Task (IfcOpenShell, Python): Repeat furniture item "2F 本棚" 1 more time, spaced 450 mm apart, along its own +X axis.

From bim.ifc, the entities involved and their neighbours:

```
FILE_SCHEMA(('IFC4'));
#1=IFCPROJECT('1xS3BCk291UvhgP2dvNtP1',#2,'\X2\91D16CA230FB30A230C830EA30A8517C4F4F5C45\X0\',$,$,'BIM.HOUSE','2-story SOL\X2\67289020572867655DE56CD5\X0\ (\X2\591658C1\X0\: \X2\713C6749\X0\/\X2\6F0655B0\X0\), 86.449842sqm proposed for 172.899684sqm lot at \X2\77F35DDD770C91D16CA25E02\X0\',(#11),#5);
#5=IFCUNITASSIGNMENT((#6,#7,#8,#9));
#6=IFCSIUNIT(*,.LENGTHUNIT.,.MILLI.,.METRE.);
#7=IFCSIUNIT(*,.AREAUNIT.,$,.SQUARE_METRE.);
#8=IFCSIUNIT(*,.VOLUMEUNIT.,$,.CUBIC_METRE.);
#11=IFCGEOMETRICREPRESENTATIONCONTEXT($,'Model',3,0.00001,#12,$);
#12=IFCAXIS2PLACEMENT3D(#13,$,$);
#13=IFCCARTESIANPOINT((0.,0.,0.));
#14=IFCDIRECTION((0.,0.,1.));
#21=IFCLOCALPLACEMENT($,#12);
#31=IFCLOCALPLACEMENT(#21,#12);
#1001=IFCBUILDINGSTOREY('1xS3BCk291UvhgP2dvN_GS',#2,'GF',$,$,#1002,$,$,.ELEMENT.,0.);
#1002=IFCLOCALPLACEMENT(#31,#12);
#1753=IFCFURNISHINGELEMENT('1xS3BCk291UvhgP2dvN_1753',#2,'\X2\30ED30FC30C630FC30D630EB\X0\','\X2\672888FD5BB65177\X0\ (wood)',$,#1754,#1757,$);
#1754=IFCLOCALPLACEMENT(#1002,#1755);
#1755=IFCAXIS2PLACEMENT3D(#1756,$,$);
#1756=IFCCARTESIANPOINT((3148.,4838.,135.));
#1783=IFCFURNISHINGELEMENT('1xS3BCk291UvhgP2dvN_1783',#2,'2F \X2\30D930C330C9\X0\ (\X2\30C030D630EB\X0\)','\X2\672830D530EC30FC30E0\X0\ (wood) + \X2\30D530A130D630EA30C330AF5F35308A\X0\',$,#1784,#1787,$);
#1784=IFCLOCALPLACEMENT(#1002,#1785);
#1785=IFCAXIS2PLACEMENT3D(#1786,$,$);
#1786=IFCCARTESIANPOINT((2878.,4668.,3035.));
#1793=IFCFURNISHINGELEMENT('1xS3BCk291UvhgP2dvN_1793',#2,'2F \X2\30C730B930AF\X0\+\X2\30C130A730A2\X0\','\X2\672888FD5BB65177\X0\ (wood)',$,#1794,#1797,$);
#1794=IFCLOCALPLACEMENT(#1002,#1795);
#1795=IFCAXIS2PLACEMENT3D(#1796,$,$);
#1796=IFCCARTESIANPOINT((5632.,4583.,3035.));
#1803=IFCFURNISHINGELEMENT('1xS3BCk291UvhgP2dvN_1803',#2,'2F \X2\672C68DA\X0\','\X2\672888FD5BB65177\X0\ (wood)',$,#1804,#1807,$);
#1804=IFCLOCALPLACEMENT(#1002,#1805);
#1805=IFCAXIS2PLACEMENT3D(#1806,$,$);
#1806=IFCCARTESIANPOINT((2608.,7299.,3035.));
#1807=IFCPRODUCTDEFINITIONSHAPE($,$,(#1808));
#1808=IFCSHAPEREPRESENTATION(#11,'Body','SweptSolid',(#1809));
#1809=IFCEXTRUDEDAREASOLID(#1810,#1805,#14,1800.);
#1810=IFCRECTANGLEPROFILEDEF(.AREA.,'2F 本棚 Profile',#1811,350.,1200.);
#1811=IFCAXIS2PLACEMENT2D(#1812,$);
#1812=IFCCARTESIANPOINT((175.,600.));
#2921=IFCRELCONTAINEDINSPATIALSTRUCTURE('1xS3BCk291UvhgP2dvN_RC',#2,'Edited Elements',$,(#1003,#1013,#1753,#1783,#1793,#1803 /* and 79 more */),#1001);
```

```python
import ifcopenshell
import ifcopenshell.api.geometry
import ifcopenshell.api.root
import ifcopenshell.util.element
import ifcopenshell.util.placement
import ifcopenshell.util.unit

model = ifcopenshell.open("bim.ifc")
unit_scale = ifcopenshell.util.unit.calculate_unit_scale(model)


def reuse_history(source, copy):
    """copy_class also copies each property set's owner history, people and application; keep the originals."""
    for rel in copy.IsDefinedBy:
        if rel.is_a("IfcRelDefinesByProperties") and (history := rel.RelatingPropertyDefinition.OwnerHistory):
            rel.RelatingPropertyDefinition.OwnerHistory = source.OwnerHistory
            ifcopenshell.util.element.remove_deep2(model, history)


source = model.by_guid("1xS3BCk291UvhgP2dvN_1803")
base = ifcopenshell.util.placement.get_local_placement(source.ObjectPlacement)
step = base[:3, 0] * 0.45 / unit_scale

for i in range(1, 2):
    copy = ifcopenshell.api.root.copy_class(model, product=source)
    copy.Representation = ifcopenshell.util.element.copy_deep(
        model, source.Representation, exclude=["IfcGeometricRepresentationContext", "IfcRepresentationMap"]
    )
    reuse_history(source, copy)
    matrix = base.copy()
    matrix[:3, 3] += i * step
    print("added at", matrix[:3, 3].round(3) + 0.0)
    ifcopenshell.api.geometry.edit_object_placement(model, product=copy, matrix=matrix, is_si=False)

model.write("bim_rev.ifc")
```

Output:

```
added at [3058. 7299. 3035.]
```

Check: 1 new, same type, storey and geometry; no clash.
